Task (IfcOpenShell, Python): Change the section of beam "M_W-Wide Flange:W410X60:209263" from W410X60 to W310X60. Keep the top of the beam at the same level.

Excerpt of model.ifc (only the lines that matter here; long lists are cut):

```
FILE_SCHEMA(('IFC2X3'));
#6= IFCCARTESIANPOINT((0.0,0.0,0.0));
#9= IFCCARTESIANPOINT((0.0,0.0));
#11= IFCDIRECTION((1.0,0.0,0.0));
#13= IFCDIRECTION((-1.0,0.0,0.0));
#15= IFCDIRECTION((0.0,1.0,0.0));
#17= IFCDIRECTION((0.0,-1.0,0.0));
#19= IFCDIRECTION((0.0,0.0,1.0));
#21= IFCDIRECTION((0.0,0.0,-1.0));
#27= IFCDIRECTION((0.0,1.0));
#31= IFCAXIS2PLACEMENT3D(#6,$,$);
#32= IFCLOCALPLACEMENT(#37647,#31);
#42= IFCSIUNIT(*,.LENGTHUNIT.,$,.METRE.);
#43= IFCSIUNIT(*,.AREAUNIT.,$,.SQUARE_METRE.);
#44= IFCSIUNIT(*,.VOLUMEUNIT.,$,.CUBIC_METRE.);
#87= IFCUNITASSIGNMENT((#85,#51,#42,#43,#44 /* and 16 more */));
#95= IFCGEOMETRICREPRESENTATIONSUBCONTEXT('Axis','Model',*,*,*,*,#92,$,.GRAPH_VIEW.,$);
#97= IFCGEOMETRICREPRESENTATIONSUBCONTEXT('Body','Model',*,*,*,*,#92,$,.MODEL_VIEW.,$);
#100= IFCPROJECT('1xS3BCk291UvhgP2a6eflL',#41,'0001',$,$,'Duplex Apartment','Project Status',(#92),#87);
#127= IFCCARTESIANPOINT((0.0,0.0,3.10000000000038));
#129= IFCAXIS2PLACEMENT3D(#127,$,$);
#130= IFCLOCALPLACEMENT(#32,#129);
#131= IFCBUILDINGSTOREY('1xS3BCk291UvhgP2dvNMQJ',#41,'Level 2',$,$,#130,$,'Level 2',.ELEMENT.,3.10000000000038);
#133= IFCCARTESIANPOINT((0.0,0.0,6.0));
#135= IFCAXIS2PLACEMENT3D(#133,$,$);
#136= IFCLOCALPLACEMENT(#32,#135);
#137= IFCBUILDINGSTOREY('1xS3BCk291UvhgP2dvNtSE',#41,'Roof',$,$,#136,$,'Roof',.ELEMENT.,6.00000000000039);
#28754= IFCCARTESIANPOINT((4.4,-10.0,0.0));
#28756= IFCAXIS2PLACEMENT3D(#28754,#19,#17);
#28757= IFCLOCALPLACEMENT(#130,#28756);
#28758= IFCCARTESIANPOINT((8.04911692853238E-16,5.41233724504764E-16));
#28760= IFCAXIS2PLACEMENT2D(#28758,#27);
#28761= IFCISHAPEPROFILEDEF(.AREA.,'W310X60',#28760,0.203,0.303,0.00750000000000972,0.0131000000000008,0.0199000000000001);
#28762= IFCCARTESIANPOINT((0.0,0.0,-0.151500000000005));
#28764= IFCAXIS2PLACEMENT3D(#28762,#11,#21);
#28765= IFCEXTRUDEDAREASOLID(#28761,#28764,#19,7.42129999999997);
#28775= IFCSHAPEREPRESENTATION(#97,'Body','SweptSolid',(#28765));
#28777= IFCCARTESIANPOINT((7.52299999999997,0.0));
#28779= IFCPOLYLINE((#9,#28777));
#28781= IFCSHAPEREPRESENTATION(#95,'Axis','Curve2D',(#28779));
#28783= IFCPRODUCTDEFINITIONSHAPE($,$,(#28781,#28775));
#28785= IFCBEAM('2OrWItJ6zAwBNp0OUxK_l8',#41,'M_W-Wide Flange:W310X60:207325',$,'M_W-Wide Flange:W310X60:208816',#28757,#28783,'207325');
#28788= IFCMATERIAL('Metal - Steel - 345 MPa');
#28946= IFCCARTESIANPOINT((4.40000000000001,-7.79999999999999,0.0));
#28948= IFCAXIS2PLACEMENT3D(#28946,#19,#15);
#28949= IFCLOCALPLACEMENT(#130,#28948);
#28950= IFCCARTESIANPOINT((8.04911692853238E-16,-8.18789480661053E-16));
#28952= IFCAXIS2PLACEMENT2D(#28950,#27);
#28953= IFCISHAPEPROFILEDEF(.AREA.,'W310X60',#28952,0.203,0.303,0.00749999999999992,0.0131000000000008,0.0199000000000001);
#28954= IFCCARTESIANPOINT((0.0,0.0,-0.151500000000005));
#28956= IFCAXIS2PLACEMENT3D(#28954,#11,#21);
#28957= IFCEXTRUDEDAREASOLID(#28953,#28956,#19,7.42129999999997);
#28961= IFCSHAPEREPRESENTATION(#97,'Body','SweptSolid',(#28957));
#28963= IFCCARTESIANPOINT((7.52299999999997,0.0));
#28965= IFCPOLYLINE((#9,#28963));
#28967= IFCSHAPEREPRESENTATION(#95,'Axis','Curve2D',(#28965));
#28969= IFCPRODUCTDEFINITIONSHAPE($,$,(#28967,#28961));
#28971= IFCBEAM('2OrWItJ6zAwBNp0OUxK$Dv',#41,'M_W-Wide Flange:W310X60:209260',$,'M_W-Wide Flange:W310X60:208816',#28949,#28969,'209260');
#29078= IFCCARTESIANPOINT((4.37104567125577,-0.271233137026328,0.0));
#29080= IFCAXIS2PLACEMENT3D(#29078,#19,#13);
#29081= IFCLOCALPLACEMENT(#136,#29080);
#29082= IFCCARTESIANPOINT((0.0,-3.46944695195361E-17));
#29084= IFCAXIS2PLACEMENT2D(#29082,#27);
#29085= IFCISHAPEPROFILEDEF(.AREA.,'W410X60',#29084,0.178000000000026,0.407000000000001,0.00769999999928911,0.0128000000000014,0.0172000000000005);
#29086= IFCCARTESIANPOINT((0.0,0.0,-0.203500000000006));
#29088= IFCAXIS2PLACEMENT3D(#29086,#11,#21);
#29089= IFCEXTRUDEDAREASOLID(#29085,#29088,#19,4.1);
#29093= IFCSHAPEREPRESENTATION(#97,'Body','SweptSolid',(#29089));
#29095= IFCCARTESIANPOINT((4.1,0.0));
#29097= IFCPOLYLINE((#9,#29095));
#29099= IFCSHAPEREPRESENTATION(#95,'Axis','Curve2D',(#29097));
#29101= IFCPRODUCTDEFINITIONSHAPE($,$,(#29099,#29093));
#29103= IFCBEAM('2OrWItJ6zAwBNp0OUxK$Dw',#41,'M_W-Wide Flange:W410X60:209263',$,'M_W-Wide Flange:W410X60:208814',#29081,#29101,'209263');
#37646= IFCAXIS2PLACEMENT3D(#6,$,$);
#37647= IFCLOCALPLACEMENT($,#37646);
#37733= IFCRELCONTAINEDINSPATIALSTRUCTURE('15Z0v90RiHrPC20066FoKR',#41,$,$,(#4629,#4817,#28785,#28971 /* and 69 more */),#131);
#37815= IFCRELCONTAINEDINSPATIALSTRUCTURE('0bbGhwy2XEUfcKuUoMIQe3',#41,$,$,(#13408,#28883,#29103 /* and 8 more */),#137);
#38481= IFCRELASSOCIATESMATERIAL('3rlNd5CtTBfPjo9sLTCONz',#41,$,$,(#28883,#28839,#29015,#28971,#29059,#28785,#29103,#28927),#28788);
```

```python
import ifcopenshell
import ifcopenshell.util.element
import ifcopenshell.util.representation

model = ifcopenshell.open("model.ifc")

member = model.by_guid("2OrWItJ6zAwBNp0OUxK$Dw")
source = next(p for p in model.by_type("IfcIShapeProfileDef") if p.ProfileName == "W310X60")

body = ifcopenshell.util.representation.get_representation(member, "Model", "Body")
solid = body.Items[0]
old_profile = solid.SweptArea

# Copy the section's sizes but keep this member's own profile position.
profile = ifcopenshell.util.element.copy(model, source)
# Profiles are centred, so shift by half the change in depth to hold the top.
shift = (old_profile.OverallDepth - profile.OverallDepth) / 2
x, y = old_profile.Position.Location.Coordinates
up = (-1.0, 0.0)  # upwards, in the solid's own plane
location = model.createIfcCartesianPoint((x + up[0] * shift, y + up[1] * shift))
profile.Position = model.createIfcAxis2Placement2D(location, old_profile.Position.RefDirection)
solid.SweptArea = profile
if not model.get_total_inverses(old_profile):
    ifcopenshell.util.element.remove_deep2(model, old_profile)
member.Name = member.Name.replace("W410X60", "W310X60")
member.ObjectType = member.ObjectType.replace("W410X60", "W310X60")

print(solid.SweptArea)

model.write("model_updated.ifc")
```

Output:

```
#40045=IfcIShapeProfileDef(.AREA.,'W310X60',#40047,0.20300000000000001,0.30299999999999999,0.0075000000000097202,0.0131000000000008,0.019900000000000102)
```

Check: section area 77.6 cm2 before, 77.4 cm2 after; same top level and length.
